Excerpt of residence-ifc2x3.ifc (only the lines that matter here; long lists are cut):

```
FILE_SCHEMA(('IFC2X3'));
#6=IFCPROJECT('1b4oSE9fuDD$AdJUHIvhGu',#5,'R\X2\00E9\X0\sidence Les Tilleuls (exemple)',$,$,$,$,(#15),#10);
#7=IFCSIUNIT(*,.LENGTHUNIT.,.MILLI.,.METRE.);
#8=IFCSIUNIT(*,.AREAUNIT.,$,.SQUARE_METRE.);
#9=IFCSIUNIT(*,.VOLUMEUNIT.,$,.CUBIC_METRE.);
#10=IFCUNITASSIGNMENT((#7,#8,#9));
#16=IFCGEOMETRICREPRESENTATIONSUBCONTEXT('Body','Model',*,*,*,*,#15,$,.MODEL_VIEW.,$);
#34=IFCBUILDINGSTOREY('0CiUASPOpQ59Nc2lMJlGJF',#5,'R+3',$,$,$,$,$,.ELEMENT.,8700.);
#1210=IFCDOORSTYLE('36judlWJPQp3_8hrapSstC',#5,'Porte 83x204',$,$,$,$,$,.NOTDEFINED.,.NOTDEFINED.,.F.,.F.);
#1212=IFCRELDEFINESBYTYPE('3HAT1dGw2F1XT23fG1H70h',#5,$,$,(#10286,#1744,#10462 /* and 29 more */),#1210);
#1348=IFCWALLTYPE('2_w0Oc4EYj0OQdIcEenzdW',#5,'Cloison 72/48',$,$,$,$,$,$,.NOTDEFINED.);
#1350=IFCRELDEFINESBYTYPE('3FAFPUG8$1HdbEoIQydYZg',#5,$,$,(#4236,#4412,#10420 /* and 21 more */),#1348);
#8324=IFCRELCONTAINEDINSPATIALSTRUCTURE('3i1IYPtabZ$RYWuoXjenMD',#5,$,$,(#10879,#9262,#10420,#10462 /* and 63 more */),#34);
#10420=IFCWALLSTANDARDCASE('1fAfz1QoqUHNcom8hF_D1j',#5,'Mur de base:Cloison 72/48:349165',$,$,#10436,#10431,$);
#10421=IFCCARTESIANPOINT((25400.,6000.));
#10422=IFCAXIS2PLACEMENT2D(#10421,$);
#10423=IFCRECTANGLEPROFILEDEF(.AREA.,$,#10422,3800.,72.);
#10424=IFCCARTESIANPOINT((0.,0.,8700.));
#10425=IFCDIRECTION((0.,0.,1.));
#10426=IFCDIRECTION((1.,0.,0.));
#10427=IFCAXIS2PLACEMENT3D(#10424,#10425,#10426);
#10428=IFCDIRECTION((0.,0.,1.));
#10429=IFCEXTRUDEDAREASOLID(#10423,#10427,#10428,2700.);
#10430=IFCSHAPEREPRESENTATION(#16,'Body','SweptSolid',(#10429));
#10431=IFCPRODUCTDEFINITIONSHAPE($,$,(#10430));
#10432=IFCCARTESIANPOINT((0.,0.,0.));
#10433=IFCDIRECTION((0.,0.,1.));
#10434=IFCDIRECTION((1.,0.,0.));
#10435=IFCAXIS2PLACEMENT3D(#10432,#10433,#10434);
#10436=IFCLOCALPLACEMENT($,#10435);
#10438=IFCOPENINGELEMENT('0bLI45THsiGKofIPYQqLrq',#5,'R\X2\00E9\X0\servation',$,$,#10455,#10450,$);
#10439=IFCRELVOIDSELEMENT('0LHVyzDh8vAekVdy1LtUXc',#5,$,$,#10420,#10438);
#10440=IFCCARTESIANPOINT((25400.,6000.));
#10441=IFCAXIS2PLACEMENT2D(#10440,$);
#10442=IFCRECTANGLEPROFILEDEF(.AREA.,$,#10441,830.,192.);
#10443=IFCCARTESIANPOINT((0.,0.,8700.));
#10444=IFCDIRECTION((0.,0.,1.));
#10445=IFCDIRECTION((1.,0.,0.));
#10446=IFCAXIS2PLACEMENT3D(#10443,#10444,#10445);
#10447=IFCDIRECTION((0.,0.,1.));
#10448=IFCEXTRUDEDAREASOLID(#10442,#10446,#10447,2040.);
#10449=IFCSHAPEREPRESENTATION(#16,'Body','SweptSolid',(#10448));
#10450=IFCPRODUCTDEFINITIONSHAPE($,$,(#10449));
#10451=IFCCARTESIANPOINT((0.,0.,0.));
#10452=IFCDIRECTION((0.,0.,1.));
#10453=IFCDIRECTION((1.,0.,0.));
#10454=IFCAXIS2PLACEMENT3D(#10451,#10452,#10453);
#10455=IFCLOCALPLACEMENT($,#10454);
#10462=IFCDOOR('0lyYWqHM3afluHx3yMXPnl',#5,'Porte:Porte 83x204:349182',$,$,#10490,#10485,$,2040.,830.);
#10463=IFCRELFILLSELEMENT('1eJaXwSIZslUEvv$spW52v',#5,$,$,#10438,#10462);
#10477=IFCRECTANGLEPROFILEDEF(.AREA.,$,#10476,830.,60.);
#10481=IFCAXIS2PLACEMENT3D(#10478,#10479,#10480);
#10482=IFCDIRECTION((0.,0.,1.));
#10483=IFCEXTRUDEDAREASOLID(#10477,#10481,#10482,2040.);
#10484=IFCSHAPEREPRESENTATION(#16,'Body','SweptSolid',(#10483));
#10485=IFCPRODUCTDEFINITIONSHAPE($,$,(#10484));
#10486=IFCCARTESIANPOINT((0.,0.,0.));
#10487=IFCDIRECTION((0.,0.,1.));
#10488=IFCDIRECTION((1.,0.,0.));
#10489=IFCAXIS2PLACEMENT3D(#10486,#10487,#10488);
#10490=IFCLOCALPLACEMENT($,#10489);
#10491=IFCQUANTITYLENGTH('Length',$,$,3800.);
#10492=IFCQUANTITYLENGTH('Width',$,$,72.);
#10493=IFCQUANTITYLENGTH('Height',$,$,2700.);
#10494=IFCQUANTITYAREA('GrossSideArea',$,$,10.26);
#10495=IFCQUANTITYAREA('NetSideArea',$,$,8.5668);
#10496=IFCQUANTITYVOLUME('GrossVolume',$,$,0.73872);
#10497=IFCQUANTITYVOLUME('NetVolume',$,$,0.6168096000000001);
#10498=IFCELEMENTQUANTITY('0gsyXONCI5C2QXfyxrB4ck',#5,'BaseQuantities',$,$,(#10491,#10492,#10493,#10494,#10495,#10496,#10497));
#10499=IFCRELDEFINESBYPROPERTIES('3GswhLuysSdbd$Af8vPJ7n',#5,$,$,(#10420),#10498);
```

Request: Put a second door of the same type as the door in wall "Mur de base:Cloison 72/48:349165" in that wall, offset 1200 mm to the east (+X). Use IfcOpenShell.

```python
import ifcopenshell
import ifcopenshell.api.feature
import ifcopenshell.api.geometry
import ifcopenshell.api.pset
import ifcopenshell.api.root
import ifcopenshell.geom
import ifcopenshell.util.element
import ifcopenshell.util.placement
import ifcopenshell.util.shape
import ifcopenshell.util.unit

model = ifcopenshell.open("residence-ifc2x3.ifc")
unit_scale = ifcopenshell.util.unit.calculate_unit_scale(model)
area_scale = ifcopenshell.util.unit.calculate_unit_scale(model, "AREAUNIT")
volume_scale = ifcopenshell.util.unit.calculate_unit_scale(model, "VOLUMEUNIT")
settings = ifcopenshell.geom.settings()


def volume(element):
    """Net volume in cubic metres, openings subtracted."""
    shape = ifcopenshell.geom.create_shape(settings, element)
    return ifcopenshell.util.shape.get_volume(shape.geometry)


def reuse_history(source, copy):
    """copy_class also copies each property set's owner history, people and application; keep the originals."""
    for rel in copy.IsDefinedBy:
        if rel.is_a("IfcRelDefinesByProperties") and (history := rel.RelatingPropertyDefinition.OwnerHistory):
            rel.RelatingPropertyDefinition.OwnerHistory = source.OwnerHistory
            ifcopenshell.util.element.remove_deep2(model, history)


door = model.by_guid("0lyYWqHM3afluHx3yMXPnl")
opening = door.FillsVoids[0].RelatingOpeningElement
wall = opening.VoidsElements[0].RelatingBuildingElement
before = volume(wall)
shift = ifcopenshell.util.placement.get_local_placement(wall.ObjectPlacement)[:3, 0] * 1.2 / unit_scale

# copy_class copies the void relationship, type, container and properties, but no geometry.
new_opening = ifcopenshell.api.root.copy_class(model, product=opening)
new_opening.Representation = ifcopenshell.util.element.copy_deep(
    model, opening.Representation, exclude=["IfcGeometricRepresentationContext", "IfcRepresentationMap"]
)
reuse_history(opening, new_opening)
new_door = ifcopenshell.api.root.copy_class(model, product=door)
new_door.Representation = ifcopenshell.util.element.copy_deep(
    model, door.Representation, exclude=["IfcGeometricRepresentationContext", "IfcRepresentationMap"]
)
new_door.Name = "Porte:Porte 83x204"
reuse_history(door, new_door)
fills = ifcopenshell.api.feature.add_filling(model, opening=new_opening, element=new_door)
fills.OwnerHistory = new_door.OwnerHistory  # required in IFC2X3

for old, new in ((opening, new_opening), (door, new_door)):
    matrix = ifcopenshell.util.placement.get_local_placement(old.ObjectPlacement)
    matrix[:3, 3] += shift
    ifcopenshell.api.geometry.edit_object_placement(model, product=new, matrix=matrix, is_si=False)

after = volume(wall)
thickness = 0.072  # wall thickness in metres

# Update the wall's stored quantities.
qto = model.by_id(ifcopenshell.util.element.get_pset(wall, "BaseQuantities", should_inherit=False)["id"])
ifcopenshell.api.pset.edit_qto(model, qto=qto, properties={
    "NetSideArea": after / thickness / area_scale,
    "NetVolume": after / volume_scale,
})

print(f"wall volume {before:.3f} -> {after:.3f} m3")

model.write("residence-ifc2x3_updated.ifc")
```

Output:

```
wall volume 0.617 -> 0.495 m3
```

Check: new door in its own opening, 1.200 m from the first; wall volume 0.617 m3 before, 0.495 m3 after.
